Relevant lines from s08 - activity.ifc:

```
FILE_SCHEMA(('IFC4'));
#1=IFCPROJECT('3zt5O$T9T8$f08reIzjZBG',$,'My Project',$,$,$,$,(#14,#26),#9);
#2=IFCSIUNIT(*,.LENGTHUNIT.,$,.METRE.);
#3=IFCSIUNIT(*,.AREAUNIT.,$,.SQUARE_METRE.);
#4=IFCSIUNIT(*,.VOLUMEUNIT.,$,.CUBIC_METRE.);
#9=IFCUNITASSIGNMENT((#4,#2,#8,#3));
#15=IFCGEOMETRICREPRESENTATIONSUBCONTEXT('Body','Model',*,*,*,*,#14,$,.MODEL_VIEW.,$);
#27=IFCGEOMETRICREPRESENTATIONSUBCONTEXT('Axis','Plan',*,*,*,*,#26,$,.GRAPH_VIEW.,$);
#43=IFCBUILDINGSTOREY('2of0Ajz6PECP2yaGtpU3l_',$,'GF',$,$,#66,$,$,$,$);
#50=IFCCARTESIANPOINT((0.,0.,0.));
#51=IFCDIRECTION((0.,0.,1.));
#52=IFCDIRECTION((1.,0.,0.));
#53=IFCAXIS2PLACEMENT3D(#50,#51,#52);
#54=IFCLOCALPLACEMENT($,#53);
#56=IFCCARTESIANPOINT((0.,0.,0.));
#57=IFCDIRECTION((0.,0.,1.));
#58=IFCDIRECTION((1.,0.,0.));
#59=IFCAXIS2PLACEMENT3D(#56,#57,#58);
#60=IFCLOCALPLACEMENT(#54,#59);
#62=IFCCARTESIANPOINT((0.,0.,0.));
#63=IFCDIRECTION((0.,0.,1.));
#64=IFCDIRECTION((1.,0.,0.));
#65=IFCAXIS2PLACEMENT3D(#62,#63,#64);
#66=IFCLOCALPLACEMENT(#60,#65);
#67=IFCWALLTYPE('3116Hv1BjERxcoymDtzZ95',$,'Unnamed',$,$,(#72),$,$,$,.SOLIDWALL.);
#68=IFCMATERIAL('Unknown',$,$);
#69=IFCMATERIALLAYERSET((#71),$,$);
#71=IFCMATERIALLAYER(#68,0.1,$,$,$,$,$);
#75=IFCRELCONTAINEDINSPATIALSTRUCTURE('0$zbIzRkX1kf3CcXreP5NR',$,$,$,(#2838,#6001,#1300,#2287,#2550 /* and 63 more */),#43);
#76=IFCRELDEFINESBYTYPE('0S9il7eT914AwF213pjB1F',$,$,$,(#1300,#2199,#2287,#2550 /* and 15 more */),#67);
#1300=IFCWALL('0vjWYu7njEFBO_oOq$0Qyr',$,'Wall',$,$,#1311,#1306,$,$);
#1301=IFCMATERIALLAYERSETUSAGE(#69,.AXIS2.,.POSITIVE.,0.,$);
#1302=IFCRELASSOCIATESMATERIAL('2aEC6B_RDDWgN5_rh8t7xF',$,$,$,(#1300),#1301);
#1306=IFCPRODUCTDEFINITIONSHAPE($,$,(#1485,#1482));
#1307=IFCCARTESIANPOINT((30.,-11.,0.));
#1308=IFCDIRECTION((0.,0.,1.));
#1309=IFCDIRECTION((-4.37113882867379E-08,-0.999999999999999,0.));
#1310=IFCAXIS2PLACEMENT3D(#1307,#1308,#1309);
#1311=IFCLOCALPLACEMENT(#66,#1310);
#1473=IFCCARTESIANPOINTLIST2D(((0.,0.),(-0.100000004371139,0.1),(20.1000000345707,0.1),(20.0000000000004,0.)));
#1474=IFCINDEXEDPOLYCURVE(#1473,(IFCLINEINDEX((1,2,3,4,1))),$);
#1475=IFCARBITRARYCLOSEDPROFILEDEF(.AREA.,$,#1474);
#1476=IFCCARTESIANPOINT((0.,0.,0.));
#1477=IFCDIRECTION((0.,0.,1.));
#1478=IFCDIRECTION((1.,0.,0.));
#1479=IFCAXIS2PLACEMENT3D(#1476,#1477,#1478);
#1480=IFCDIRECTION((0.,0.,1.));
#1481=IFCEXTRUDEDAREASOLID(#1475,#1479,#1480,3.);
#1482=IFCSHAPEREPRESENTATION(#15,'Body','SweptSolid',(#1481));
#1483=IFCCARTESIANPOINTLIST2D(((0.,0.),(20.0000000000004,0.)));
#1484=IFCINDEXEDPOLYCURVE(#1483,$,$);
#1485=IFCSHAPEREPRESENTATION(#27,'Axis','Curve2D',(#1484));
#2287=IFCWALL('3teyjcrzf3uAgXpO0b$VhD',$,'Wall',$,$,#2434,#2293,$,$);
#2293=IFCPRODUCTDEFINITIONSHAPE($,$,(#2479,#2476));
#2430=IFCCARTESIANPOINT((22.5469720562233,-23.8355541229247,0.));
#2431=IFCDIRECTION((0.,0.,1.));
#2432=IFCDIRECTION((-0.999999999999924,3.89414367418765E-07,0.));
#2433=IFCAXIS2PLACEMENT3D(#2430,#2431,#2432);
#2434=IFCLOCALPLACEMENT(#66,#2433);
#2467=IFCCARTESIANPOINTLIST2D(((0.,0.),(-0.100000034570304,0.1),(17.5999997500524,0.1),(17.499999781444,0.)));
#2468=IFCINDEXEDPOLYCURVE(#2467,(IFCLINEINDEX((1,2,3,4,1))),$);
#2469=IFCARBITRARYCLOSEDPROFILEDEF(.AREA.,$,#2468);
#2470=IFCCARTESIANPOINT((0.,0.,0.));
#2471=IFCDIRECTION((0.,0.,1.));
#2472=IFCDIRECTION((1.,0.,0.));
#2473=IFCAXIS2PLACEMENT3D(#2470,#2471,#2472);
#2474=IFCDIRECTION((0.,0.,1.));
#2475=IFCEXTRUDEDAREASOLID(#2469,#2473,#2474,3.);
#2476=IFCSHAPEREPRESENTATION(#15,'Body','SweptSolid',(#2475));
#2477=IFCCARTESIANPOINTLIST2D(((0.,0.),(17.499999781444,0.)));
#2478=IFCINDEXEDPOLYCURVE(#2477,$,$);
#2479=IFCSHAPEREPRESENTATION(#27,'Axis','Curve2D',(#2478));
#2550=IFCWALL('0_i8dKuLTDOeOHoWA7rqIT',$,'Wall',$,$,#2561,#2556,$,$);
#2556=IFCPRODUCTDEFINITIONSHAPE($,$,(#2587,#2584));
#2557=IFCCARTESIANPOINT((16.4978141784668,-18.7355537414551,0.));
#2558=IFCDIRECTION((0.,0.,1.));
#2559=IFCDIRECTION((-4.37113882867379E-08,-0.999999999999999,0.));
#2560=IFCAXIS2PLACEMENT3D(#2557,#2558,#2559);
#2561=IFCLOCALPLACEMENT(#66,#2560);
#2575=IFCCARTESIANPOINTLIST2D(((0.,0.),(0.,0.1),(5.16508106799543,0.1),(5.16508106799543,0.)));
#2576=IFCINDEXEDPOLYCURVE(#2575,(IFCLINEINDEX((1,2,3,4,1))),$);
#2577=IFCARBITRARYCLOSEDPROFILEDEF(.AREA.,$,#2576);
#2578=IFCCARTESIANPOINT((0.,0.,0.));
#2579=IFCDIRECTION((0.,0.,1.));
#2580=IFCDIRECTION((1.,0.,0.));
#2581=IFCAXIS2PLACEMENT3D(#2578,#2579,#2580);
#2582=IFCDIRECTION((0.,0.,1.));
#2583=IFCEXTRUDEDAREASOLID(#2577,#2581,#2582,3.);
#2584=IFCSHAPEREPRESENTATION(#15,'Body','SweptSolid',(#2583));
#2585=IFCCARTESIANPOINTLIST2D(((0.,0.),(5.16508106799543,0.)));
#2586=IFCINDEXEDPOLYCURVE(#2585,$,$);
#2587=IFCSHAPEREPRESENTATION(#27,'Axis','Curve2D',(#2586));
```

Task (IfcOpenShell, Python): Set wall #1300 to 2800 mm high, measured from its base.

```python
import ifcopenshell
import ifcopenshell.geom
import ifcopenshell.util.representation
import ifcopenshell.util.shape
import ifcopenshell.util.unit

model = ifcopenshell.open("s08 - activity.ifc")
unit_scale = ifcopenshell.util.unit.calculate_unit_scale(model)
settings = ifcopenshell.geom.settings()


def volume(element):
    """Net volume in cubic metres, openings subtracted."""
    shape = ifcopenshell.geom.create_shape(settings, element)
    return ifcopenshell.util.shape.get_volume(shape.geometry)


wall = model.by_guid("0vjWYu7njEFBO_oOq$0Qyr")
before = volume(wall)

body = ifcopenshell.util.representation.get_representation(wall, "Model", "Body")
solid = body.Items[0]
old_height = solid.Depth
solid.Depth = 2.8 / unit_scale
after = volume(wall)

print(f"height {old_height:g} -> {solid.Depth:g}, volume {before:.3f} -> {after:.3f} m3")

model.write("s08 - activity_edited.ifc")
```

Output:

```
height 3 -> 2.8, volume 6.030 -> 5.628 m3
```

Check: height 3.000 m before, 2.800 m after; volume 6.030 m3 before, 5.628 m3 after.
